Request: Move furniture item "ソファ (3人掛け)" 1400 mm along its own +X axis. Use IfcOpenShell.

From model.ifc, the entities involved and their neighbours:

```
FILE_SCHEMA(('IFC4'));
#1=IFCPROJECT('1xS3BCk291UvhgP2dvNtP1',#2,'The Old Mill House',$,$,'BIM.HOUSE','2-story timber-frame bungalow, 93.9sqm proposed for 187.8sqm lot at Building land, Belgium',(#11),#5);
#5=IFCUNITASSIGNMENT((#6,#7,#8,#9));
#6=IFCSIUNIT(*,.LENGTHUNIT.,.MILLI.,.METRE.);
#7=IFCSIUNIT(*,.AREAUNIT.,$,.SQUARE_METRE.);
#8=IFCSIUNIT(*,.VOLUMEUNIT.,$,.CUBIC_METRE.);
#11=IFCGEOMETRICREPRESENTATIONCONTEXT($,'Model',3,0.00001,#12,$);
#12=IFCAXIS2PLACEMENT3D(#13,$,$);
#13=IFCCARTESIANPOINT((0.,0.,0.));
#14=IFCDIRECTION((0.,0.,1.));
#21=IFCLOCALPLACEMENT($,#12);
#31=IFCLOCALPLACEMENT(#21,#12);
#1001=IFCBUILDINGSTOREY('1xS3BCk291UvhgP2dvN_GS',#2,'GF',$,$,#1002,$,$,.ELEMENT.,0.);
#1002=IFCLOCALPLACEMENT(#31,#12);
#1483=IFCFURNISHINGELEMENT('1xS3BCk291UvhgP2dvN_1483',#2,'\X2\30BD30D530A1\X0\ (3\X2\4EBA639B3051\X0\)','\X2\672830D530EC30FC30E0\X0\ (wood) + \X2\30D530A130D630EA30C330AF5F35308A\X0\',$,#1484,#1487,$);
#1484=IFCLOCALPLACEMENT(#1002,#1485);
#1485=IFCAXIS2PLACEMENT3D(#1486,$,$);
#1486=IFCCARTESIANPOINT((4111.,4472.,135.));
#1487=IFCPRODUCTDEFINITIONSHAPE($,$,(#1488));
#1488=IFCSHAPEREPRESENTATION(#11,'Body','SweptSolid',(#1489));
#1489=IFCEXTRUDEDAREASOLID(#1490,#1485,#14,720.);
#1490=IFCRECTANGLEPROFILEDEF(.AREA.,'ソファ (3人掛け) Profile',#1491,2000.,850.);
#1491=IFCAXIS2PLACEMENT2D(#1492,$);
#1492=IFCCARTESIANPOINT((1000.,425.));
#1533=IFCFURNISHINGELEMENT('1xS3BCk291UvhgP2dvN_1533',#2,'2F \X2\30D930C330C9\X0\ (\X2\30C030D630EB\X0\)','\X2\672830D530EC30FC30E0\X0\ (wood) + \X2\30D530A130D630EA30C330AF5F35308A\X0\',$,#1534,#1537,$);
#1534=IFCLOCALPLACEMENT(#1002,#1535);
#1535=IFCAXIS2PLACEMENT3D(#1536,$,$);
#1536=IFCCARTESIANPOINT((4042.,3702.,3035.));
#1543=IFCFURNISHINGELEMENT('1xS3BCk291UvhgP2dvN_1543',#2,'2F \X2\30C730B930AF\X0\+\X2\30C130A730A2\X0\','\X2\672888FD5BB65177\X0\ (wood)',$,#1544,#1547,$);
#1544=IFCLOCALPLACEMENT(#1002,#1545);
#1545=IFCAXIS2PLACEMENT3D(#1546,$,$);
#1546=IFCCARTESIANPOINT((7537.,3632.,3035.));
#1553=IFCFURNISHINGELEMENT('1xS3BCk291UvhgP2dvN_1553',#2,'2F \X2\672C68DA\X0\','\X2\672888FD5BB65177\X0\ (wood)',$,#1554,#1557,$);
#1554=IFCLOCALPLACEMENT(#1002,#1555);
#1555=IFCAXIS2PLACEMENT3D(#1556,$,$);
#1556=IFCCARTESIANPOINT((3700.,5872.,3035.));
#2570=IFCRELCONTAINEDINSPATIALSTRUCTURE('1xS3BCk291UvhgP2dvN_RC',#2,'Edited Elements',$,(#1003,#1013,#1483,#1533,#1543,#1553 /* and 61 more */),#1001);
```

```python
import ifcopenshell
import ifcopenshell.api.geometry
import ifcopenshell.util.placement

model = ifcopenshell.open("model.ifc")

item = model.by_guid("1xS3BCk291UvhgP2dvN_1483")
matrix = ifcopenshell.util.placement.get_local_placement(item.ObjectPlacement)
matrix[:3, 3] += matrix[:3, 0] * 1400.0
ifcopenshell.api.geometry.edit_object_placement(model, product=item, matrix=matrix, is_si=False)

print(ifcopenshell.util.placement.get_local_placement(item.ObjectPlacement).round(3) + 0.0)

model.write("model_rev.ifc")
```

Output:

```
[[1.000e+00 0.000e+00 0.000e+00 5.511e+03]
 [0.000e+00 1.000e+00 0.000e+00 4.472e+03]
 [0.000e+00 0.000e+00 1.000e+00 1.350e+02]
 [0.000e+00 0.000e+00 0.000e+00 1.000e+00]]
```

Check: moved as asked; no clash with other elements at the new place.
